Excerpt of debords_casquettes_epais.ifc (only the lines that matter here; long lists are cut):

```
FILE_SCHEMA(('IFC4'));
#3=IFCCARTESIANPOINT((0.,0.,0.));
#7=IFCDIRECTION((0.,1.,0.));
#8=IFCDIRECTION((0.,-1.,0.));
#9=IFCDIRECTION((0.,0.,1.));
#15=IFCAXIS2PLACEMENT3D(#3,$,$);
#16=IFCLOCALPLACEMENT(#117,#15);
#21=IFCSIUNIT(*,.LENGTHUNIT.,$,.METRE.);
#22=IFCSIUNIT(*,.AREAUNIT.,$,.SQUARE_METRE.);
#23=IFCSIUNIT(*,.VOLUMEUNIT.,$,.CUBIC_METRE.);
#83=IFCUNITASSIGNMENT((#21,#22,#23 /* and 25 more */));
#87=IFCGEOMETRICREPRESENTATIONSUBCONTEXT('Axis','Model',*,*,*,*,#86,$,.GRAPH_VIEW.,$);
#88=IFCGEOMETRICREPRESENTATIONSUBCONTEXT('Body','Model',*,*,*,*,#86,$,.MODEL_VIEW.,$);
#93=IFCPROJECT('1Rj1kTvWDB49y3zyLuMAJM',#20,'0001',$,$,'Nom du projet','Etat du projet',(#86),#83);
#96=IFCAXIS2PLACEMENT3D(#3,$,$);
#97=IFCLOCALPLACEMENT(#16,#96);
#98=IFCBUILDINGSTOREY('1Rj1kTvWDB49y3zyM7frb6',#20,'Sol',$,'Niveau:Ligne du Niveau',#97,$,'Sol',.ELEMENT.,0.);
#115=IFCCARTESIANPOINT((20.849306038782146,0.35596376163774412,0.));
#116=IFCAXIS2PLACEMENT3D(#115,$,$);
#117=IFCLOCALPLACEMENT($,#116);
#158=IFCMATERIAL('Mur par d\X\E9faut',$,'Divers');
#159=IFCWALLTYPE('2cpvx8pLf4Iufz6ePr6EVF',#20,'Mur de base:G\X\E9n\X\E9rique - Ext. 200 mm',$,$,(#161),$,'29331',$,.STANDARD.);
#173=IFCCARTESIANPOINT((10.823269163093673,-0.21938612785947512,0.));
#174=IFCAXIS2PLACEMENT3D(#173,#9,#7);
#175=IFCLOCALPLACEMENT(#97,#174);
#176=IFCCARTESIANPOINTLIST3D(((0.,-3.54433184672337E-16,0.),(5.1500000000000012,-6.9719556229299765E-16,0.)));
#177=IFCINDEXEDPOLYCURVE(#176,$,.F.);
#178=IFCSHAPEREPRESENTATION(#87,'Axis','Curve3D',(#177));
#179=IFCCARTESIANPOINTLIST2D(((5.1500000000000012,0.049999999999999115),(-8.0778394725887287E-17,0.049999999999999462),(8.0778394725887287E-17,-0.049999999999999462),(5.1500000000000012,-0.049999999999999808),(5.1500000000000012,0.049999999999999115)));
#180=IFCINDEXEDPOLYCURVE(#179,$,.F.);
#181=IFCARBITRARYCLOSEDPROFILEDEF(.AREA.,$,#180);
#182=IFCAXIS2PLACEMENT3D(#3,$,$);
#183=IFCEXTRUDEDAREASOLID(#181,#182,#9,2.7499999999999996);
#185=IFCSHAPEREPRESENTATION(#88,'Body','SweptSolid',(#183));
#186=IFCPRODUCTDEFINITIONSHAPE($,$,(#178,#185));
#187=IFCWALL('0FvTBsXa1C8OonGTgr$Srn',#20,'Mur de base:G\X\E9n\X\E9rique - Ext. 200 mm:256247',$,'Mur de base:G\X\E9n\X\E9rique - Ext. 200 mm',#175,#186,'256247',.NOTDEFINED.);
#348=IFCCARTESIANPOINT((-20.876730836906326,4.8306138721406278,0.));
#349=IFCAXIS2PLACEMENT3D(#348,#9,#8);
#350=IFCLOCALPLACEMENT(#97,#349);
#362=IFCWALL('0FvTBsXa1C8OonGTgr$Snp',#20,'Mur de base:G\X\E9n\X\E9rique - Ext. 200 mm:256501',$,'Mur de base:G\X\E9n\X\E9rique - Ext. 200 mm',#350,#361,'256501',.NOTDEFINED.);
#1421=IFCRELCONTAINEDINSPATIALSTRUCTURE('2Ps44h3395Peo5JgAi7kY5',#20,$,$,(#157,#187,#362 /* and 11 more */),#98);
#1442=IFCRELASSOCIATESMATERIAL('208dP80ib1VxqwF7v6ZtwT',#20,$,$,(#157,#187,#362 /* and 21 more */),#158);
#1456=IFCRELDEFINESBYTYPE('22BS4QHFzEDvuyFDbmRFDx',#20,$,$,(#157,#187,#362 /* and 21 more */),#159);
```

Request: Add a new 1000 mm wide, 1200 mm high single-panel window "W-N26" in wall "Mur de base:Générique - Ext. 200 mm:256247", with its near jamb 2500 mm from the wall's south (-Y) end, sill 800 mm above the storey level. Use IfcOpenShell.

```python
import numpy as np
import ifcopenshell
import ifcopenshell.api.feature
import ifcopenshell.api.geometry
import ifcopenshell.api.root
import ifcopenshell.api.spatial
import ifcopenshell.geom
import ifcopenshell.util.element
import ifcopenshell.util.placement
import ifcopenshell.util.representation
import ifcopenshell.util.shape
import ifcopenshell.util.unit

model = ifcopenshell.open("debords_casquettes_epais.ifc")
unit_scale = ifcopenshell.util.unit.calculate_unit_scale(model)
settings = ifcopenshell.geom.settings()


def volume(element):
    """Net volume in cubic metres, openings subtracted."""
    shape = ifcopenshell.geom.create_shape(settings, element)
    return ifcopenshell.util.shape.get_volume(shape.geometry)


wall = model.by_guid("0FvTBsXa1C8OonGTgr$Srn")
storey = ifcopenshell.util.element.get_container(wall, ifc_class="IfcBuildingStorey")
context = ifcopenshell.util.representation.get_context(model, "Model", "Body", "MODEL_VIEW")
before = volume(wall)

width, height, from_end, sill = 1, 1.2, 2.5, 0.8  # metres

# The wall runs along its own X axis, and the end named is its -X end.
wall_shape = ifcopenshell.geom.create_shape(settings, wall)
x, y, z = ifcopenshell.util.shape.get_vertices(wall_shape.geometry).T
start = x.min() + from_end
face, thickness = float(y.min()), float(y.max() - y.min())
wall_matrix = ifcopenshell.util.placement.get_local_placement(wall.ObjectPlacement)
level = ifcopenshell.util.placement.get_local_placement(storey.ObjectPlacement)[2, 3]


def in_wall(x, y):
    """Placement at x, y metres in the wall's axes, at sill height."""
    matrix = wall_matrix.copy()
    matrix[:, 3] = wall_matrix @ np.array([x / unit_scale, y / unit_scale, 0.0, 1.0])
    matrix[2, 3] = level + sill / unit_scale
    return matrix


# Opening: a box that overshoots both wall faces by 50 mm.
opening = ifcopenshell.api.root.create_entity(model, ifc_class="IfcOpeningElement", predefined_type="OPENING")
box = ifcopenshell.api.geometry.add_wall_representation(
    model, context=context, length=width, height=height, thickness=thickness + 0.1
)
ifcopenshell.api.geometry.assign_representation(model, product=opening, representation=box)
ifcopenshell.api.geometry.edit_object_placement(model, product=opening, matrix=in_wall(start, face - 0.05), is_si=False)
ifcopenshell.api.feature.add_feature(model, feature=opening, element=wall)

window = ifcopenshell.api.root.create_entity(model, ifc_class="IfcWindow", name="W-N26", predefined_type="WINDOW")
window.OverallWidth, window.OverallHeight = width / unit_scale, height / unit_scale
window.PartitioningType = "SINGLE_PANEL"
body = ifcopenshell.api.geometry.add_window_representation(
    model,
    context=context,
    overall_width=window.OverallWidth,
    overall_height=window.OverallHeight,
    partition_type="SINGLE_PANEL",
)
ifcopenshell.api.geometry.assign_representation(model, product=window, representation=body)
ifcopenshell.api.spatial.assign_container(model, products=[window], relating_structure=storey)
ifcopenshell.api.feature.add_filling(model, opening=opening, element=window)

# Centre the window in the wall's thickness.
ifcopenshell.api.geometry.edit_object_placement(model, product=window, matrix=in_wall(start, face), is_si=False)
window_shape = ifcopenshell.geom.create_shape(settings, window)
depth = ifcopenshell.util.shape.get_vertices(window_shape.geometry)[:, 1]
offset = face + thickness / 2 - (depth.min() + depth.max()) / 2
ifcopenshell.api.geometry.edit_object_placement(model, product=window, matrix=in_wall(start, offset), is_si=False)

after = volume(wall)

print(f"wall volume {before:.3f} -> {after:.3f} m3")

model.write("debords_casquettes_epais_edited.ifc")
```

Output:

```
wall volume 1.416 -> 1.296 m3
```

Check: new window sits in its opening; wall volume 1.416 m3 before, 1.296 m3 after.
